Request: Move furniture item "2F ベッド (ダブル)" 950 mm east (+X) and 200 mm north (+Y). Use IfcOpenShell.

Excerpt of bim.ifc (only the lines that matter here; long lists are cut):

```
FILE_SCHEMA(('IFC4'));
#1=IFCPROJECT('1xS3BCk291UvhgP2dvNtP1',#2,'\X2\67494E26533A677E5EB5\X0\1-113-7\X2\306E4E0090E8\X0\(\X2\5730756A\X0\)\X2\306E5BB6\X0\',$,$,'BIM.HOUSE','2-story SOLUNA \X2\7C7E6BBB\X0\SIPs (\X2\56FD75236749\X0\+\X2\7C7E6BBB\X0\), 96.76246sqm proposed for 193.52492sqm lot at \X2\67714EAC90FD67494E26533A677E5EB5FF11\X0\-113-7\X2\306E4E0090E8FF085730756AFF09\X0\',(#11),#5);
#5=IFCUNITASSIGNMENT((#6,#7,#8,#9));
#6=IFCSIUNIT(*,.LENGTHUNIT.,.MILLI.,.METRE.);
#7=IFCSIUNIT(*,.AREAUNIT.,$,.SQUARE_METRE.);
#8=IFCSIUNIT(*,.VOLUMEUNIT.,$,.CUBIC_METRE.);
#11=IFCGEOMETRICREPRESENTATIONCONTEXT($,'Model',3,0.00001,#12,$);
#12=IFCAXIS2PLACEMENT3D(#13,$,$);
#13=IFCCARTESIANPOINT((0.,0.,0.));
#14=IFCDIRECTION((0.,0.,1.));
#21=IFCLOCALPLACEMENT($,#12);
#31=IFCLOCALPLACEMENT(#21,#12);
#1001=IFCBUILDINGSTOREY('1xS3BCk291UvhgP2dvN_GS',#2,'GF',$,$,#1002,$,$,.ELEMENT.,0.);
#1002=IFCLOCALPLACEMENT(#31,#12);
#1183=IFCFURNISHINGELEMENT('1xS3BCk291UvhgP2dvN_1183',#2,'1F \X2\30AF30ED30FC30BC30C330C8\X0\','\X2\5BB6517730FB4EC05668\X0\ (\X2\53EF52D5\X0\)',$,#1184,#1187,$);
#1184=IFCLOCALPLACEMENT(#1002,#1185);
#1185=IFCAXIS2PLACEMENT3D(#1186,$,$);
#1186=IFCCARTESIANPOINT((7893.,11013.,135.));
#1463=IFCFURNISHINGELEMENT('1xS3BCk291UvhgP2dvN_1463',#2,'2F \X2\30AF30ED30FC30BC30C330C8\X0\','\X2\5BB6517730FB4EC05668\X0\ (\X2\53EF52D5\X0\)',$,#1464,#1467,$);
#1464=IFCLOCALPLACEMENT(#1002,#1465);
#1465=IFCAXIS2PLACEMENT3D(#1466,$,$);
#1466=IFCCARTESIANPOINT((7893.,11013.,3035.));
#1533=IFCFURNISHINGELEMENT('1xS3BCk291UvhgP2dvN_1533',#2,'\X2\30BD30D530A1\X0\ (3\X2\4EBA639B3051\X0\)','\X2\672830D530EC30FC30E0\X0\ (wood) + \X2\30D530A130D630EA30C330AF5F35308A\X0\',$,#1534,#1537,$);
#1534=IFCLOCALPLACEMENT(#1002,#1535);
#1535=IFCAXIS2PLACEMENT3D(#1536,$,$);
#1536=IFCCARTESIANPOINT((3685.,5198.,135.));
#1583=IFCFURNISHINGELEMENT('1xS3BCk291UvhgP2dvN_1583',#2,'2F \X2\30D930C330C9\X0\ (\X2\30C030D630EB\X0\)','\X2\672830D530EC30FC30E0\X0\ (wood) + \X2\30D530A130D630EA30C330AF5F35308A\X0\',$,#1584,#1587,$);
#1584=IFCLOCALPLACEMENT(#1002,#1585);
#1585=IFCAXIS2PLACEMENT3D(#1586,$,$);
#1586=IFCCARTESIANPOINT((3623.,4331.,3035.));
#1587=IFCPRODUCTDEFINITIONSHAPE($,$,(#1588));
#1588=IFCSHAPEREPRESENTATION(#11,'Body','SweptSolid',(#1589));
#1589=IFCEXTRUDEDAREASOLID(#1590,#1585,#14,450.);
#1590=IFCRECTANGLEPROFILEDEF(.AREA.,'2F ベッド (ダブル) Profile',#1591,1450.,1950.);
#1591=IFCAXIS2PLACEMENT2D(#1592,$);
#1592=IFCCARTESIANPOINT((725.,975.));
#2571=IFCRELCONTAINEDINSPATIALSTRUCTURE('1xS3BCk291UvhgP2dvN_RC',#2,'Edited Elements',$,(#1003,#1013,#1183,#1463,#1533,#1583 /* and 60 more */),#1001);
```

```python
import ifcopenshell
import ifcopenshell.api.geometry
import ifcopenshell.util.placement
import ifcopenshell.util.unit

model = ifcopenshell.open("bim.ifc")
unit_scale = ifcopenshell.util.unit.calculate_unit_scale(model)

item = model.by_id(1583)
matrix = ifcopenshell.util.placement.get_local_placement(item.ObjectPlacement)
matrix[0, 3] += 0.95 / unit_scale
matrix[1, 3] += 0.2 / unit_scale
ifcopenshell.api.geometry.edit_object_placement(model, product=item, matrix=matrix, is_si=False)

print(ifcopenshell.util.placement.get_local_placement(item.ObjectPlacement).round(3) + 0.0)

model.write("bim_edited.ifc")
```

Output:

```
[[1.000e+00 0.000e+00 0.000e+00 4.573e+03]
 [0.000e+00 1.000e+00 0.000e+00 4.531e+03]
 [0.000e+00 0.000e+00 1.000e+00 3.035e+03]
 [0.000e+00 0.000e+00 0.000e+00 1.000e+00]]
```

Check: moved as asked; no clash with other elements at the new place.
